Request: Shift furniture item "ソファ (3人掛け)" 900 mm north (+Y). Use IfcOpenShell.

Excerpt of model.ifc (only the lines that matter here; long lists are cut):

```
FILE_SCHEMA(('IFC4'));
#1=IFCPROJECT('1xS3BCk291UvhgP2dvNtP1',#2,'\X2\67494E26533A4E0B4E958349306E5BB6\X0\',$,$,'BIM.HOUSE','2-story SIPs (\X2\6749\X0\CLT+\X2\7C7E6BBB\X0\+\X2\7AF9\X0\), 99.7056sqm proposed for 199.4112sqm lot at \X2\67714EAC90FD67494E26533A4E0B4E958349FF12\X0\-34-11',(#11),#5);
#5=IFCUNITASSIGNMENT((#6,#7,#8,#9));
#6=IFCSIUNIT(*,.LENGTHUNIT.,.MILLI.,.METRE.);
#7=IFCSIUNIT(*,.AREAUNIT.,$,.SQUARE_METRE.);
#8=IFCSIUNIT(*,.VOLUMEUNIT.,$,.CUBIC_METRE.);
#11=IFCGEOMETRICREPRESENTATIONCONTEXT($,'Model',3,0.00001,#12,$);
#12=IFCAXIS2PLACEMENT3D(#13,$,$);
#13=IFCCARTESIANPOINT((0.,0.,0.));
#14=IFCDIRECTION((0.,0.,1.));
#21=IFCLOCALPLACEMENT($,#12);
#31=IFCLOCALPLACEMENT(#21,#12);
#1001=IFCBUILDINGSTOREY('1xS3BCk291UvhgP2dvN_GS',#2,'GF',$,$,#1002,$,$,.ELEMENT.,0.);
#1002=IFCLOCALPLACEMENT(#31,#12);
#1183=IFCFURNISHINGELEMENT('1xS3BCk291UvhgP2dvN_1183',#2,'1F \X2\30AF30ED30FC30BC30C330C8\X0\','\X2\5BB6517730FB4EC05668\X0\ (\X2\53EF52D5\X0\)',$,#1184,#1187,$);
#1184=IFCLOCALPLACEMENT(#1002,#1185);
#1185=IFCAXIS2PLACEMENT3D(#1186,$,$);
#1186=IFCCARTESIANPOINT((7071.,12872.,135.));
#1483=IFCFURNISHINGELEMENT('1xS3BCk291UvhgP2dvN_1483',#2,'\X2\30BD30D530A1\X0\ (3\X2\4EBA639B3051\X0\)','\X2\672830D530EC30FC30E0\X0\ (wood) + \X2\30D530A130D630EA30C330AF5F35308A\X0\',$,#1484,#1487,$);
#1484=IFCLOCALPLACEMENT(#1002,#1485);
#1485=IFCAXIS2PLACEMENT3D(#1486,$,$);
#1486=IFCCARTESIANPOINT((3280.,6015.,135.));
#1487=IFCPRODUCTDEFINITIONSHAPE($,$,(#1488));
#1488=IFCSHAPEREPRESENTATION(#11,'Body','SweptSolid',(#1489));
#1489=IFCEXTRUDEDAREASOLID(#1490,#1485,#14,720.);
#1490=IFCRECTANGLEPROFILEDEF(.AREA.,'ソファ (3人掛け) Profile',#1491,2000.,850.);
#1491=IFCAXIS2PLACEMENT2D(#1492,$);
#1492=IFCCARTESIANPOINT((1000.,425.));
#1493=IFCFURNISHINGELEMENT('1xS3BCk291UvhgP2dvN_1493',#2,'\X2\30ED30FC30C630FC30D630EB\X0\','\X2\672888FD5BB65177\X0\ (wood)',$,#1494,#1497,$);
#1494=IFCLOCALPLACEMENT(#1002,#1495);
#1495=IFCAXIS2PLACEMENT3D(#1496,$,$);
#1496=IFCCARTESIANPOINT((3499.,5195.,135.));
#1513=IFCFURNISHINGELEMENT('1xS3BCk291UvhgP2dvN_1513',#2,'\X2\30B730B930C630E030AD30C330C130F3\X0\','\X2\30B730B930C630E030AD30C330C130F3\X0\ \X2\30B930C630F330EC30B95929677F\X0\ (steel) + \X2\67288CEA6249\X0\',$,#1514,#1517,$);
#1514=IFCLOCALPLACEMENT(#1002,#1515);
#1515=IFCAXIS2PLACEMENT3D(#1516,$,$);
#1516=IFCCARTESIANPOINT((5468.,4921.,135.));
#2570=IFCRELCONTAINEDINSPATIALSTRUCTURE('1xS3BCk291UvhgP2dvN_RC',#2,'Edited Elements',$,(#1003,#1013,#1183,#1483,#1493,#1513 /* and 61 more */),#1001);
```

```python
import ifcopenshell
import ifcopenshell.api.geometry
import ifcopenshell.util.placement
import ifcopenshell.util.unit

model = ifcopenshell.open("model.ifc")
unit_scale = ifcopenshell.util.unit.calculate_unit_scale(model)

item = model.by_guid("1xS3BCk291UvhgP2dvN_1483")
matrix = ifcopenshell.util.placement.get_local_placement(item.ObjectPlacement)
matrix[1, 3] += 0.9 / unit_scale
ifcopenshell.api.geometry.edit_object_placement(model, product=item, matrix=matrix, is_si=False)

print(ifcopenshell.util.placement.get_local_placement(item.ObjectPlacement).round(3) + 0.0)

model.write("model_v2.ifc")
```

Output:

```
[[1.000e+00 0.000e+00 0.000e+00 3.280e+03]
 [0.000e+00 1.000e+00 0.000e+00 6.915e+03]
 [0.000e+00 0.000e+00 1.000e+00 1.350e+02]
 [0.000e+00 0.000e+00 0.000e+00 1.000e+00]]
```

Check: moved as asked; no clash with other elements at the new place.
